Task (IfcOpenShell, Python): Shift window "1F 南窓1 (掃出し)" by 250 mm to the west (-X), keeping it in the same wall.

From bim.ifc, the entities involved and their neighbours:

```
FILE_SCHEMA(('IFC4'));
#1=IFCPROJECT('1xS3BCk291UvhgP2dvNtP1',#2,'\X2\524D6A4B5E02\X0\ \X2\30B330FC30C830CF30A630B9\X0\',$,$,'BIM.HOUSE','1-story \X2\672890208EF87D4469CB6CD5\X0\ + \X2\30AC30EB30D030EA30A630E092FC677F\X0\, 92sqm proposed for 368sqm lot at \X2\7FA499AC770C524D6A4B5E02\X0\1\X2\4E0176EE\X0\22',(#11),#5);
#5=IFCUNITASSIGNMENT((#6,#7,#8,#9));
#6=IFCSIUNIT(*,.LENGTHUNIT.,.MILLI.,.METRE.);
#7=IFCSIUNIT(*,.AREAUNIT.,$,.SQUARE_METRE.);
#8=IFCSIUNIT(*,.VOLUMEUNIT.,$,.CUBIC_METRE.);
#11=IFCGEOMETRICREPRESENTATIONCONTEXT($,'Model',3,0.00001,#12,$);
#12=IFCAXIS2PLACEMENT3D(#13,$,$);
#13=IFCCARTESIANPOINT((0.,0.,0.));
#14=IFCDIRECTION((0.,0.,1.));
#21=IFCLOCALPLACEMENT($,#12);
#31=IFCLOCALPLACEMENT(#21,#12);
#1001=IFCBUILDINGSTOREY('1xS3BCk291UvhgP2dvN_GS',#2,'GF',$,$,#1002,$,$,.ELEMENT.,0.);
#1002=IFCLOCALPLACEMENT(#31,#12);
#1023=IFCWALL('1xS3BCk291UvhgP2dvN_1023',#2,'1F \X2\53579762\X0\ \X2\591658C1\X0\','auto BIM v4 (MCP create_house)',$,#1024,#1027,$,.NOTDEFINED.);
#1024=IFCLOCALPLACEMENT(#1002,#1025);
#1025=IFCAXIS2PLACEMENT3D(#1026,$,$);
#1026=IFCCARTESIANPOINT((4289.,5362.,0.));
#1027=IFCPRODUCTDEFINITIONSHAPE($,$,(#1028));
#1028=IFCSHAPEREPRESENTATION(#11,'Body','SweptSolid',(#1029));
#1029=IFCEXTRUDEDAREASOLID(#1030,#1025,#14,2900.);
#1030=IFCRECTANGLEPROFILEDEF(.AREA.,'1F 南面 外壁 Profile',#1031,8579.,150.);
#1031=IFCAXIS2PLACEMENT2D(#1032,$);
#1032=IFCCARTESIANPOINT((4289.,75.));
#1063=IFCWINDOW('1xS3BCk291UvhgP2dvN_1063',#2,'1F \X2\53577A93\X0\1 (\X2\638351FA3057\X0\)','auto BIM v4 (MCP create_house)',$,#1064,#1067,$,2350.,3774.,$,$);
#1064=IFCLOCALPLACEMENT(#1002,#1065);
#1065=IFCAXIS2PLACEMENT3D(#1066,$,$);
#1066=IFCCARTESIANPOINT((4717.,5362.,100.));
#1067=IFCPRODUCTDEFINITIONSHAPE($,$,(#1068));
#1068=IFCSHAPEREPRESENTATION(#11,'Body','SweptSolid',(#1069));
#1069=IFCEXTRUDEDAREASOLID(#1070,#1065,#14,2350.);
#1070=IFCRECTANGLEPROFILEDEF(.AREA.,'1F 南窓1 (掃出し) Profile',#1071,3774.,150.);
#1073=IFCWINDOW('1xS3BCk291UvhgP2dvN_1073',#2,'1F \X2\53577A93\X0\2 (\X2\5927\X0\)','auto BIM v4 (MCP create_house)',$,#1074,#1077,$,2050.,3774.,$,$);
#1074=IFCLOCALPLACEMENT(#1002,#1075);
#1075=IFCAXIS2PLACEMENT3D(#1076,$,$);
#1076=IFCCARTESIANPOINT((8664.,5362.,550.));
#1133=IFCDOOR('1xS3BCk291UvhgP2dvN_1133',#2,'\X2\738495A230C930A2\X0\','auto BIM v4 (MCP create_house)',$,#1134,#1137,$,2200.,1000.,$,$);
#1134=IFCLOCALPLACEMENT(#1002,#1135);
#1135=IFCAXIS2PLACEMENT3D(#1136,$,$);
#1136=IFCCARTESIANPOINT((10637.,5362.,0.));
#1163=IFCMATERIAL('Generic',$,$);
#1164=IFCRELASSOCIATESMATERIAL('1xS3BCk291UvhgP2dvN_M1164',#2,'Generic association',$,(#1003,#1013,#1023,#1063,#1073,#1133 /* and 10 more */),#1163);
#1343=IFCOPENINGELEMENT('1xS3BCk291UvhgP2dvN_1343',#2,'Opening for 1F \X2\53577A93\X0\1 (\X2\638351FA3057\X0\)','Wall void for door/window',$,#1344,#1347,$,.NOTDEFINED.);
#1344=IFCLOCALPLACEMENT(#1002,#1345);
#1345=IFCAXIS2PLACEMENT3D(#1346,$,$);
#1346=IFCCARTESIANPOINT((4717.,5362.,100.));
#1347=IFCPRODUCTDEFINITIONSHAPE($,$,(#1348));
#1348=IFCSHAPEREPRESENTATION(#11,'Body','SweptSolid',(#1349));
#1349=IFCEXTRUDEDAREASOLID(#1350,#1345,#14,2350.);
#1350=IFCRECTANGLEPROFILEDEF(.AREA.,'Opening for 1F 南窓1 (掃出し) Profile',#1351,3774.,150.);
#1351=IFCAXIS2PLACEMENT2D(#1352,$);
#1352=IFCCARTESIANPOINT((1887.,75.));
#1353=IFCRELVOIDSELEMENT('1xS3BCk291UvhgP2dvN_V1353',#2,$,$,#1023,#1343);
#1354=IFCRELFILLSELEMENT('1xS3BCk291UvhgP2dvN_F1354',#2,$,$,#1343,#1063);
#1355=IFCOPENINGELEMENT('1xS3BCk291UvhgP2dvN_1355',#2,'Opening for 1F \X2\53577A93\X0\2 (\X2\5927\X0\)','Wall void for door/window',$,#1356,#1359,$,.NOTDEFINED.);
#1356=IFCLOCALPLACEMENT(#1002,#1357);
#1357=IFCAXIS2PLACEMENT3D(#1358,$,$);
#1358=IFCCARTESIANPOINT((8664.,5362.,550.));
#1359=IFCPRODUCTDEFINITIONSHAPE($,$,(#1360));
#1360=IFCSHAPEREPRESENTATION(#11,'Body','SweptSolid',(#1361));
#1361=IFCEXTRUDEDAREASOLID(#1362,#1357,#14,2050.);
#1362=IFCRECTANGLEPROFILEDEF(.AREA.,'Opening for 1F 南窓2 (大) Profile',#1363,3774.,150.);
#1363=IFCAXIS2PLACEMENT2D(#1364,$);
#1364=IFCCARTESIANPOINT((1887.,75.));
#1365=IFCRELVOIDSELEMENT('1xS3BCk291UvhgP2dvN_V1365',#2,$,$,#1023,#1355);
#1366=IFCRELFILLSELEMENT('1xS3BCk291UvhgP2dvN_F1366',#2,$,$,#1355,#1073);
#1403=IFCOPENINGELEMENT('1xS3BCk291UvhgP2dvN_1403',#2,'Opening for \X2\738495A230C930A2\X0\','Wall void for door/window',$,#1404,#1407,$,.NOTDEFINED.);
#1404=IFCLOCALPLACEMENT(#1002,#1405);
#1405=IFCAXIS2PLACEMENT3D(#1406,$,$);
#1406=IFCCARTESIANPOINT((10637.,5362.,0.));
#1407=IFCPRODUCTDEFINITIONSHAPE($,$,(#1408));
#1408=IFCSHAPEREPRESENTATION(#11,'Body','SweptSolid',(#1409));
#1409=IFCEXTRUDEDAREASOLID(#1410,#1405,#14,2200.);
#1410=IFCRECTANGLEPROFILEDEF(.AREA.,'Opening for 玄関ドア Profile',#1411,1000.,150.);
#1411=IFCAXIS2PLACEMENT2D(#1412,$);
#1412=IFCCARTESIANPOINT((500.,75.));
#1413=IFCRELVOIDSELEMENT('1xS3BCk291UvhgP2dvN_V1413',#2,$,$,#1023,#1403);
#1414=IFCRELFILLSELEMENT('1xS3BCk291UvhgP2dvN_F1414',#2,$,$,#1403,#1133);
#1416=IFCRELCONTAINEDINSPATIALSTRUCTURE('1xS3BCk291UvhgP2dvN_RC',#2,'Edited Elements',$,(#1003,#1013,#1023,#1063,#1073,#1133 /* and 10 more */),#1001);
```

```python
import ifcopenshell
import ifcopenshell.api.geometry
import ifcopenshell.util.placement

model = ifcopenshell.open("bim.ifc")

window = model.by_guid("1xS3BCk291UvhgP2dvN_1063")
opening = window.FillsVoids[0].RelatingOpeningElement
wall = opening.VoidsElements[0].RelatingBuildingElement

wall_matrix = ifcopenshell.util.placement.get_local_placement(wall.ObjectPlacement)
shift = wall_matrix[:3, 0] * -250.0
before = ifcopenshell.util.placement.get_local_placement(window.ObjectPlacement)[:3, 3].copy()

# The window is not placed relative to its opening, so move both.
for product in (opening, window):
    matrix = ifcopenshell.util.placement.get_local_placement(product.ObjectPlacement)
    matrix[:3, 3] += shift
    ifcopenshell.api.geometry.edit_object_placement(model, product=product, matrix=matrix, is_si=False)

after = ifcopenshell.util.placement.get_local_placement(window.ObjectPlacement)[:3, 3]
print("window moved by", (after - before).round(3) + 0.0)

model.write("bim_v2.ifc")
```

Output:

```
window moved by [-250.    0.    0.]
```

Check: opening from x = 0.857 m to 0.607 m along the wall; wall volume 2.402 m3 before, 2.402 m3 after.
